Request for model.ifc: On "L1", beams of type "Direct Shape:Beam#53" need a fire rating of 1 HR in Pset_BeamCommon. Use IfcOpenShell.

First a look at what the model holds.

```python
import ifcopenshell
import ifcopenshell.util.element

model = ifcopenshell.open("model.ifc")
print(model.schema)
storey = next(s for s in model.by_type("IfcBuildingStorey") if s.Name == "L1")
beams = [e for e in ifcopenshell.util.element.get_decomposition(storey) if e.is_a("IfcBeam")]
seen = {}
for e in beams:
    element_type = ifcopenshell.util.element.get_type(e)
    key = (element_type.Name if element_type != e and element_type else None, ifcopenshell.util.element.get_pset(e, "Pset_BeamCommon", "FireRating"))
    seen[key] = seen.get(key, 0) + 1
for (name, value), count in sorted(seen.items(), key=str):
    print(count, "x", name, "|", value)
```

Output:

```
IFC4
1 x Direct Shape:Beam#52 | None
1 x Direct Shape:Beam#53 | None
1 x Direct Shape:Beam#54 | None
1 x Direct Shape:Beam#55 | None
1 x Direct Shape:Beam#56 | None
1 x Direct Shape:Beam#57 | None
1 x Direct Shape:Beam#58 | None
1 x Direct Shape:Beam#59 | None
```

```python
import ifcopenshell
import ifcopenshell.api.pset
import ifcopenshell.util.element

model = ifcopenshell.open("model.ifc")

storey = next(s for s in model.by_type("IfcBuildingStorey") if s.Name == "L1")
beams = [e for e in ifcopenshell.util.element.get_decomposition(storey) if e.is_a("IfcBeam")]

count = 0
for e in beams:
    element_type = ifcopenshell.util.element.get_type(e)
    if element_type in (None, e) or element_type.Name != "Direct Shape:Beam#53":
        continue
    # add_pset returns the element's existing set when there is one.
    pset = ifcopenshell.api.pset.add_pset(model, product=e, name="Pset_BeamCommon")
    ifcopenshell.api.pset.edit_pset(model, pset=pset, properties={"FireRating": "1 HR"})
    count += 1

print(count, "beams updated")

model.write("model_rev.ifc")
```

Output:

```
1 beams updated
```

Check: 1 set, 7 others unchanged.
